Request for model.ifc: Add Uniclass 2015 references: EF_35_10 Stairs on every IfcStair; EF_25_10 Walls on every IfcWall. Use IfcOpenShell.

First a look at what the model holds.

```python
import ifcopenshell

model = ifcopenshell.open("model.ifc")
print(model.schema)
print("classifications:", [c.Name for c in model.by_type("IfcClassification")])
for ifc_class in ("IfcDoor", "IfcRoof", "IfcStair", "IfcWall", "IfcWindow"):
    print(ifc_class, len(model.by_type(ifc_class)))
```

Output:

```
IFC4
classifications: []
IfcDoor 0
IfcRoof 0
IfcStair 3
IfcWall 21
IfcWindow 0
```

```python
import ifcopenshell
import ifcopenshell.api.classification

model = ifcopenshell.open("model.ifc")

system = ifcopenshell.api.classification.add_classification(model, classification="Uniclass 2015")

codes = {
    "IfcStair": ("EF_35_10", "Stairs"),
    "IfcWall": ("EF_25_10", "Walls"),
}
for ifc_class, (code, name) in codes.items():
    products = model.by_type(ifc_class)
    ifcopenshell.api.classification.add_reference(
        model, products=products, classification=system, identification=code, name=name
    )
    print(code, len(products))

model.write("model_edited.ifc")
```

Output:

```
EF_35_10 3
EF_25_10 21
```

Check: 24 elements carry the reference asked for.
